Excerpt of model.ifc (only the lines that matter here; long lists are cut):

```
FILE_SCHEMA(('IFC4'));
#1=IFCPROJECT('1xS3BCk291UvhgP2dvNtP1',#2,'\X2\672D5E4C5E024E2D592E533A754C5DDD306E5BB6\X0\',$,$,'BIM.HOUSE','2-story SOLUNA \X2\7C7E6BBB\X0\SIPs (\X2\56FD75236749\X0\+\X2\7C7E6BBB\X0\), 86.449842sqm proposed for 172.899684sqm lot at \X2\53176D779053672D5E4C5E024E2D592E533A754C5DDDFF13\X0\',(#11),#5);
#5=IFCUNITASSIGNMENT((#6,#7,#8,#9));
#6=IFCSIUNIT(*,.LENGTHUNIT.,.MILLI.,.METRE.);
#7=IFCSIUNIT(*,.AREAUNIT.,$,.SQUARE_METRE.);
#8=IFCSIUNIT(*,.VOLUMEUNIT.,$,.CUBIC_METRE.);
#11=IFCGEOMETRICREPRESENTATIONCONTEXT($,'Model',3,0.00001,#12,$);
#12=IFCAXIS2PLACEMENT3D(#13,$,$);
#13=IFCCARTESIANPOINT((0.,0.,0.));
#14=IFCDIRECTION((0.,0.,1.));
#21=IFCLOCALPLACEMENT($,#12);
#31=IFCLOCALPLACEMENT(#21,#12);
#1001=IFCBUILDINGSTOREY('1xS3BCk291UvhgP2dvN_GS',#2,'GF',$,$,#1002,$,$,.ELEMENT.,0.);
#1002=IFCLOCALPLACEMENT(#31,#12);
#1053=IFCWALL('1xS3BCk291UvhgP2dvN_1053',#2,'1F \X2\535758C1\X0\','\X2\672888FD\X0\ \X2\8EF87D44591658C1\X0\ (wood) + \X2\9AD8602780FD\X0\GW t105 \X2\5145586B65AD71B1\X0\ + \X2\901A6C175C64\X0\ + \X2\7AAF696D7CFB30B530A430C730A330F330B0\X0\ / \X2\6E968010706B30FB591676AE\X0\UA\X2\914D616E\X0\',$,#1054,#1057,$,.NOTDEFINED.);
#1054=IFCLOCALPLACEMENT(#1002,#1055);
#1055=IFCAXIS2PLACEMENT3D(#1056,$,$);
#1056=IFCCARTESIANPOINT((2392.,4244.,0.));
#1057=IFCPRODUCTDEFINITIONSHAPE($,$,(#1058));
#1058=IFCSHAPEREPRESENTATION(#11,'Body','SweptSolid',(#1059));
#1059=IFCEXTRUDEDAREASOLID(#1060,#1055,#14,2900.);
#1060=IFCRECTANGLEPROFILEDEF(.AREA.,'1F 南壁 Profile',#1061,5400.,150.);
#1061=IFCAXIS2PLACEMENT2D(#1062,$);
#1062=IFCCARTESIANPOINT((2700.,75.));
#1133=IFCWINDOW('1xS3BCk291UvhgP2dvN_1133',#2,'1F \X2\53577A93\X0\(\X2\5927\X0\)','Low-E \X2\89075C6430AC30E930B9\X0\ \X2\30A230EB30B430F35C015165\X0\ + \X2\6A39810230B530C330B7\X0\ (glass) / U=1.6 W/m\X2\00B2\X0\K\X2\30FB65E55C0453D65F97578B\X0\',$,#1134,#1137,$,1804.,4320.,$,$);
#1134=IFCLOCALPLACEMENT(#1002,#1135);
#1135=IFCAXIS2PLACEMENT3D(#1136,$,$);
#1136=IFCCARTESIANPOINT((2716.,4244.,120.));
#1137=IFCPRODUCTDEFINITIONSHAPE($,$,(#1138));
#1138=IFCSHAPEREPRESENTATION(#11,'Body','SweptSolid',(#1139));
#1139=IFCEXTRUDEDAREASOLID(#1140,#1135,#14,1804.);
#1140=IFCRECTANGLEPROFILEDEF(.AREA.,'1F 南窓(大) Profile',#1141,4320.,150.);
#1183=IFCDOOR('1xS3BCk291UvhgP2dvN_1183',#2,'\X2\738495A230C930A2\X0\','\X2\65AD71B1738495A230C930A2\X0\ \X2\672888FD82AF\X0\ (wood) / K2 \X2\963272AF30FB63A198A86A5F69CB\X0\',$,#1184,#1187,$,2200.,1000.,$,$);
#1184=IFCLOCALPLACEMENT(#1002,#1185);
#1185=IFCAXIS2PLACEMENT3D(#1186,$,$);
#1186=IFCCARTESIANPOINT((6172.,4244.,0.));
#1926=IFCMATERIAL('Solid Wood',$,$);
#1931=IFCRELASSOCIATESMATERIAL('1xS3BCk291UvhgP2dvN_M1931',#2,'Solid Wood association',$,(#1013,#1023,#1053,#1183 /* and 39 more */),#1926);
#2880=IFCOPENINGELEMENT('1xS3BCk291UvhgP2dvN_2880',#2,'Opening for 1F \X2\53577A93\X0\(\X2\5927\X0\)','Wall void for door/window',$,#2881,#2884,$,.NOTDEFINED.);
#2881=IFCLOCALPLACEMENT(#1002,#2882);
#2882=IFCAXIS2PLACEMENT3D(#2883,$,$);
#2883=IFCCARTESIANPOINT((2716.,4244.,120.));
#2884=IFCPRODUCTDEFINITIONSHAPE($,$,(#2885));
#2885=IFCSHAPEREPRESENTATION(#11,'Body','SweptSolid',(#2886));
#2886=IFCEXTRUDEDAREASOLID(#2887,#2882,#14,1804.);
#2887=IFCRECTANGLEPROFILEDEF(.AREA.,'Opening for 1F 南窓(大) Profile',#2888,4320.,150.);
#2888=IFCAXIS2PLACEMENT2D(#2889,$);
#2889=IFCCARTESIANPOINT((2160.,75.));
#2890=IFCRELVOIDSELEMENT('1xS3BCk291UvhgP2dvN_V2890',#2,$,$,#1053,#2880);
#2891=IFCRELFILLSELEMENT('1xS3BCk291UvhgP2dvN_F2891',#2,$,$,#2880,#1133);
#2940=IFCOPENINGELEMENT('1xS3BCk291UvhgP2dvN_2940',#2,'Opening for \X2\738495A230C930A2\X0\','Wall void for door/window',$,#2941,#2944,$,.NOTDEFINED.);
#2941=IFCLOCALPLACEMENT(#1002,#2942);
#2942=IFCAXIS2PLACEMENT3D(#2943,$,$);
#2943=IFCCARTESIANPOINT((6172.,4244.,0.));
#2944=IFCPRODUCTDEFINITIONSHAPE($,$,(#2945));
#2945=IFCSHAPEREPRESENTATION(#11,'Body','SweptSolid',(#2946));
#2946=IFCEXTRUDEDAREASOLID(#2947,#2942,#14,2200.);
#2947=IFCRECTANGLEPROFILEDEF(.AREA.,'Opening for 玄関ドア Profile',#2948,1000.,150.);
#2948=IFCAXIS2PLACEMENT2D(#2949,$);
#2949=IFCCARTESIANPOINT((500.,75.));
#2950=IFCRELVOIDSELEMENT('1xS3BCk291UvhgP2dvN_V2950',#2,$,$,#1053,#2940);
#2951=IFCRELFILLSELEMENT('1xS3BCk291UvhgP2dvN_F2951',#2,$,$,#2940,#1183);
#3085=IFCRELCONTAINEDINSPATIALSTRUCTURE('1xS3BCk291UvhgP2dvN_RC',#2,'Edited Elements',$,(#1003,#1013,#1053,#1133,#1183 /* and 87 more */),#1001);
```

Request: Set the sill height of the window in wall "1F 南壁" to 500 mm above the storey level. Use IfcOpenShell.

```python
import numpy as np
import ifcopenshell
import ifcopenshell.api.geometry
import ifcopenshell.geom
import ifcopenshell.util.element
import ifcopenshell.util.placement
import ifcopenshell.util.shape
import ifcopenshell.util.unit

model = ifcopenshell.open("model.ifc")
unit_scale = ifcopenshell.util.unit.calculate_unit_scale(model)

window = model.by_guid("1xS3BCk291UvhgP2dvN_1133")
opening = window.FillsVoids[0].RelatingOpeningElement
storey = ifcopenshell.util.element.get_container(window, ifc_class="IfcBuildingStorey")
level = ifcopenshell.util.placement.get_local_placement(storey.ObjectPlacement)[2, 3]

# The opening's origin need not be at the sill, so measure its lowest point.
shape = ifcopenshell.geom.create_shape(ifcopenshell.geom.settings(), opening)
bottom = ifcopenshell.util.shape.get_shape_bottom_elevation(shape, shape.geometry) / unit_scale
dz = level + 0.5 / unit_scale - bottom

shift = np.array([0.0, 0.0, dz])
# The window is not placed relative to its opening, so move both.
for product in (opening, window):
    matrix = ifcopenshell.util.placement.get_local_placement(product.ObjectPlacement)
    matrix[:3, 3] += shift
    ifcopenshell.api.geometry.edit_object_placement(model, product=product, matrix=matrix, is_si=False)

print(f"moved by {dz * unit_scale:+.3f} m")

model.write("model_updated.ifc")
```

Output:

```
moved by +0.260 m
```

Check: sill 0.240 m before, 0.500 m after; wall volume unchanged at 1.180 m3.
